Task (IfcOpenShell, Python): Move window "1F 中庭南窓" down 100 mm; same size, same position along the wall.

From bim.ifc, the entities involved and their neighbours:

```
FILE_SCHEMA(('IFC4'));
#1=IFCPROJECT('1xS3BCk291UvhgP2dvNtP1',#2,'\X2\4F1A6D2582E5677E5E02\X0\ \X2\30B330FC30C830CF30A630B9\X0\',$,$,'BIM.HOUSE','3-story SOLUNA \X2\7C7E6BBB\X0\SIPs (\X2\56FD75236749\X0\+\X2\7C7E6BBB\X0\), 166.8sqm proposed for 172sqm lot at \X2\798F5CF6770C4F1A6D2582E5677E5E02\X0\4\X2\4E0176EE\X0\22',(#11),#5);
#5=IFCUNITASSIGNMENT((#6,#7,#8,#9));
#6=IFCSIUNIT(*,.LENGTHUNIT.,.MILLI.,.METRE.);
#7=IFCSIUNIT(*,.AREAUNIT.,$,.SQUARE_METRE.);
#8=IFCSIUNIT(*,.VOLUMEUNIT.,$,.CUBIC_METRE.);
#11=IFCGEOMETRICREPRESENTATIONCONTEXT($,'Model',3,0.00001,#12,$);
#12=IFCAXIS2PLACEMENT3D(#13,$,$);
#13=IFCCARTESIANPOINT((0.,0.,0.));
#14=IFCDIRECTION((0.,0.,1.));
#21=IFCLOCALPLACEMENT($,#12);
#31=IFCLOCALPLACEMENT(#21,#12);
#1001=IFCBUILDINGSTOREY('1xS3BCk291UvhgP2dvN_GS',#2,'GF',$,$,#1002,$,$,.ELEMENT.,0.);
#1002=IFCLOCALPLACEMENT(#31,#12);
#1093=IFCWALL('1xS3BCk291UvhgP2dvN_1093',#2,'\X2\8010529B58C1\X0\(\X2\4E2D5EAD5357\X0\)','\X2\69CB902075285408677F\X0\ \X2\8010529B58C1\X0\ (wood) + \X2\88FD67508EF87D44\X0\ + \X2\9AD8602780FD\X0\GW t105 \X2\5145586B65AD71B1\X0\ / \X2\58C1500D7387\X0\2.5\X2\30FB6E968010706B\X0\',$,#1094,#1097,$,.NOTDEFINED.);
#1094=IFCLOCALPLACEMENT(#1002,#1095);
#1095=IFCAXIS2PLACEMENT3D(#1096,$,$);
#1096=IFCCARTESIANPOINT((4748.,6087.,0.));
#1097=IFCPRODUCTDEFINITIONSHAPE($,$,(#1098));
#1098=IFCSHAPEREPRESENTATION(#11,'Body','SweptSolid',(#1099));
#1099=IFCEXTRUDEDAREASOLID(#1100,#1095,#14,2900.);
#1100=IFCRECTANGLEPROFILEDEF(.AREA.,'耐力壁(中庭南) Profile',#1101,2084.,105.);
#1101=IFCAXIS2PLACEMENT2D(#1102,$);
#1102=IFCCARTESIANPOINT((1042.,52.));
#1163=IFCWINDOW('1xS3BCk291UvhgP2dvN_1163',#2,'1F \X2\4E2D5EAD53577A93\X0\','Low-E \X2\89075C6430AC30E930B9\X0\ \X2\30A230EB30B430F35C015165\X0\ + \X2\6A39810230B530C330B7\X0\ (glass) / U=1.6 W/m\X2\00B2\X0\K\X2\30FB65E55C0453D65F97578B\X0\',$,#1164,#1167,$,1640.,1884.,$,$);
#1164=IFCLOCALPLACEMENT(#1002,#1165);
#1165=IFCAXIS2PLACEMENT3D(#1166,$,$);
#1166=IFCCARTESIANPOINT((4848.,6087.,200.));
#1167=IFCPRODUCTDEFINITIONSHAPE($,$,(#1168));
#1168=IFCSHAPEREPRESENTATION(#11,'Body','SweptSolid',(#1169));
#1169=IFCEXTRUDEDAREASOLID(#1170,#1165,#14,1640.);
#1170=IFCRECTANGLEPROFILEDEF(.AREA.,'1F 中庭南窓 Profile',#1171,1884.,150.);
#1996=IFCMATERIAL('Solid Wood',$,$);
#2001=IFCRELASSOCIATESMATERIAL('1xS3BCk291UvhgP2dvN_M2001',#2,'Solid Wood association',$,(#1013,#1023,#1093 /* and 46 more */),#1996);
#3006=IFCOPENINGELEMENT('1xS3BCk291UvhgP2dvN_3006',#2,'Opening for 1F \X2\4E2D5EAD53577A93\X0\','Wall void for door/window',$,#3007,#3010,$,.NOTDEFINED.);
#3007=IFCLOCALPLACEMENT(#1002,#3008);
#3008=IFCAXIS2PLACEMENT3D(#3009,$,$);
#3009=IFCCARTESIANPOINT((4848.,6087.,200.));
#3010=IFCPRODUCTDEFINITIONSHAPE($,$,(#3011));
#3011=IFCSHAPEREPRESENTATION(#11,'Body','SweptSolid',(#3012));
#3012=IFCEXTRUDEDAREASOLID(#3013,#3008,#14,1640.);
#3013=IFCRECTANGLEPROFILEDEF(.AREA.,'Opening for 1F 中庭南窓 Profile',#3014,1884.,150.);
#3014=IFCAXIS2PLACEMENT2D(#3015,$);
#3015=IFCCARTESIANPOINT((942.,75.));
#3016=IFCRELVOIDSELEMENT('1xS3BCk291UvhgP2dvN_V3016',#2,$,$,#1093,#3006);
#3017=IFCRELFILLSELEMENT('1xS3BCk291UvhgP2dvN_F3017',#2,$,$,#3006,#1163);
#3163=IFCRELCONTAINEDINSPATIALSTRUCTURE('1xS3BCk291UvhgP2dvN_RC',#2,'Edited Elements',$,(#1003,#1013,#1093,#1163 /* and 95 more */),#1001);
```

```python
import numpy as np
import ifcopenshell
import ifcopenshell.api.geometry
import ifcopenshell.util.placement
import ifcopenshell.util.unit

model = ifcopenshell.open("bim.ifc")
unit_scale = ifcopenshell.util.unit.calculate_unit_scale(model)

window = model.by_id(1163)
opening = window.FillsVoids[0].RelatingOpeningElement
dz = -0.1 / unit_scale

shift = np.array([0.0, 0.0, dz])
# The window is not placed relative to its opening, so move both.
for product in (opening, window):
    matrix = ifcopenshell.util.placement.get_local_placement(product.ObjectPlacement)
    matrix[:3, 3] += shift
    ifcopenshell.api.geometry.edit_object_placement(model, product=product, matrix=matrix, is_si=False)

print(f"moved by {dz * unit_scale:+.3f} m")

model.write("bim-out.ifc")
```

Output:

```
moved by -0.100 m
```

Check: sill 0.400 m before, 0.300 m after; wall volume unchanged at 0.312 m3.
